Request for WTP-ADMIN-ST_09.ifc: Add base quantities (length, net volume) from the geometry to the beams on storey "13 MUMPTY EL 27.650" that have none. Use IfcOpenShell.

First a look at what the model holds.

```python
import ifcopenshell
import ifcopenshell.util.element
import ifcopenshell.util.unit

model = ifcopenshell.open("WTP-ADMIN-ST_09.ifc")
print(model.schema)
for unit_type in ("LENGTHUNIT", "AREAUNIT", "VOLUMEUNIT"):
    print(unit_type, ifcopenshell.util.unit.calculate_unit_scale(model, unit_type))
storey = next(s for s in model.by_type("IfcBuildingStorey") if s.Name == "13 MUMPTY EL 27.650")
beams = [e for e in ifcopenshell.util.element.get_decomposition(storey) if e.is_a("IfcBeam")]
for e in sorted(beams, key=lambda e: e.id()):
    print(e.id(), e.is_a(), e.Name, list(ifcopenshell.util.element.get_psets(e, qtos_only=True)), sep=" | ")
```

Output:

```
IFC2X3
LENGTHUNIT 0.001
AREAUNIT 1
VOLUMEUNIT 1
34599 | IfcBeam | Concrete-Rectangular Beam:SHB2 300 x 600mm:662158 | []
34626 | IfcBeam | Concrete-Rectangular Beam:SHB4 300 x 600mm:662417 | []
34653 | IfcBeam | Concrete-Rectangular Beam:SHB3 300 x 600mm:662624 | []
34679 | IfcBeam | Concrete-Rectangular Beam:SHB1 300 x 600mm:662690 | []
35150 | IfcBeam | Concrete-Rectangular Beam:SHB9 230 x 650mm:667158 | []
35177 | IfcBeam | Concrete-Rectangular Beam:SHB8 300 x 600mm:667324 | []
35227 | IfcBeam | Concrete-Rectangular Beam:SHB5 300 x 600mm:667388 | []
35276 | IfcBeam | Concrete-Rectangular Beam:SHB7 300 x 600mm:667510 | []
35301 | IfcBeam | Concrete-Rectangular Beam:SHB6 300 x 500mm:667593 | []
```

```python
import ifcopenshell
import ifcopenshell.api.pset
import ifcopenshell.geom
import ifcopenshell.util.element
import ifcopenshell.util.shape
import ifcopenshell.util.unit

model = ifcopenshell.open("WTP-ADMIN-ST_09.ifc")
unit_scale = ifcopenshell.util.unit.calculate_unit_scale(model)
volume_scale = ifcopenshell.util.unit.calculate_unit_scale(model, "VOLUMEUNIT")
settings = ifcopenshell.geom.settings()

storey = next(s for s in model.by_type("IfcBuildingStorey") if s.Name == "13 MUMPTY EL 27.650")
beams = [e for e in ifcopenshell.util.element.get_decomposition(storey) if e.is_a("IfcBeam")]

for e in sorted(beams, key=lambda e: e.id()):
    if ifcopenshell.util.element.get_psets(e, qtos_only=True, should_inherit=False):
        continue
    # Geometry comes back in metres, in the element's own axes.
    shape = ifcopenshell.geom.create_shape(settings, e)
    values = {
        "Length": ifcopenshell.util.shape.get_max_xyz(shape.geometry) / unit_scale,
        "NetVolume": ifcopenshell.util.shape.get_volume(shape.geometry) / volume_scale,
    }
    qto = ifcopenshell.api.pset.add_qto(model, product=e, name="BaseQuantities")
    ifcopenshell.api.pset.edit_qto(model, qto=qto, properties=values)
    print(e.id(), {k: round(v, 3) for k, v in values.items()})

model.write("WTP-ADMIN-ST_09_v2.ifc")
```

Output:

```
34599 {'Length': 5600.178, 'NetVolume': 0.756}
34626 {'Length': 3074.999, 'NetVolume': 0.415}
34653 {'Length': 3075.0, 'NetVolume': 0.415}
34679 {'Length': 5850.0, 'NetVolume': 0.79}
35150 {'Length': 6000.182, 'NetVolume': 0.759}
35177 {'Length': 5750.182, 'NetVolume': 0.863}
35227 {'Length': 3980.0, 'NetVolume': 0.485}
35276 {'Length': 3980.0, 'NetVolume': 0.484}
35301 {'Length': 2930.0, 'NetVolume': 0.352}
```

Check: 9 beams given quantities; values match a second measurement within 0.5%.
